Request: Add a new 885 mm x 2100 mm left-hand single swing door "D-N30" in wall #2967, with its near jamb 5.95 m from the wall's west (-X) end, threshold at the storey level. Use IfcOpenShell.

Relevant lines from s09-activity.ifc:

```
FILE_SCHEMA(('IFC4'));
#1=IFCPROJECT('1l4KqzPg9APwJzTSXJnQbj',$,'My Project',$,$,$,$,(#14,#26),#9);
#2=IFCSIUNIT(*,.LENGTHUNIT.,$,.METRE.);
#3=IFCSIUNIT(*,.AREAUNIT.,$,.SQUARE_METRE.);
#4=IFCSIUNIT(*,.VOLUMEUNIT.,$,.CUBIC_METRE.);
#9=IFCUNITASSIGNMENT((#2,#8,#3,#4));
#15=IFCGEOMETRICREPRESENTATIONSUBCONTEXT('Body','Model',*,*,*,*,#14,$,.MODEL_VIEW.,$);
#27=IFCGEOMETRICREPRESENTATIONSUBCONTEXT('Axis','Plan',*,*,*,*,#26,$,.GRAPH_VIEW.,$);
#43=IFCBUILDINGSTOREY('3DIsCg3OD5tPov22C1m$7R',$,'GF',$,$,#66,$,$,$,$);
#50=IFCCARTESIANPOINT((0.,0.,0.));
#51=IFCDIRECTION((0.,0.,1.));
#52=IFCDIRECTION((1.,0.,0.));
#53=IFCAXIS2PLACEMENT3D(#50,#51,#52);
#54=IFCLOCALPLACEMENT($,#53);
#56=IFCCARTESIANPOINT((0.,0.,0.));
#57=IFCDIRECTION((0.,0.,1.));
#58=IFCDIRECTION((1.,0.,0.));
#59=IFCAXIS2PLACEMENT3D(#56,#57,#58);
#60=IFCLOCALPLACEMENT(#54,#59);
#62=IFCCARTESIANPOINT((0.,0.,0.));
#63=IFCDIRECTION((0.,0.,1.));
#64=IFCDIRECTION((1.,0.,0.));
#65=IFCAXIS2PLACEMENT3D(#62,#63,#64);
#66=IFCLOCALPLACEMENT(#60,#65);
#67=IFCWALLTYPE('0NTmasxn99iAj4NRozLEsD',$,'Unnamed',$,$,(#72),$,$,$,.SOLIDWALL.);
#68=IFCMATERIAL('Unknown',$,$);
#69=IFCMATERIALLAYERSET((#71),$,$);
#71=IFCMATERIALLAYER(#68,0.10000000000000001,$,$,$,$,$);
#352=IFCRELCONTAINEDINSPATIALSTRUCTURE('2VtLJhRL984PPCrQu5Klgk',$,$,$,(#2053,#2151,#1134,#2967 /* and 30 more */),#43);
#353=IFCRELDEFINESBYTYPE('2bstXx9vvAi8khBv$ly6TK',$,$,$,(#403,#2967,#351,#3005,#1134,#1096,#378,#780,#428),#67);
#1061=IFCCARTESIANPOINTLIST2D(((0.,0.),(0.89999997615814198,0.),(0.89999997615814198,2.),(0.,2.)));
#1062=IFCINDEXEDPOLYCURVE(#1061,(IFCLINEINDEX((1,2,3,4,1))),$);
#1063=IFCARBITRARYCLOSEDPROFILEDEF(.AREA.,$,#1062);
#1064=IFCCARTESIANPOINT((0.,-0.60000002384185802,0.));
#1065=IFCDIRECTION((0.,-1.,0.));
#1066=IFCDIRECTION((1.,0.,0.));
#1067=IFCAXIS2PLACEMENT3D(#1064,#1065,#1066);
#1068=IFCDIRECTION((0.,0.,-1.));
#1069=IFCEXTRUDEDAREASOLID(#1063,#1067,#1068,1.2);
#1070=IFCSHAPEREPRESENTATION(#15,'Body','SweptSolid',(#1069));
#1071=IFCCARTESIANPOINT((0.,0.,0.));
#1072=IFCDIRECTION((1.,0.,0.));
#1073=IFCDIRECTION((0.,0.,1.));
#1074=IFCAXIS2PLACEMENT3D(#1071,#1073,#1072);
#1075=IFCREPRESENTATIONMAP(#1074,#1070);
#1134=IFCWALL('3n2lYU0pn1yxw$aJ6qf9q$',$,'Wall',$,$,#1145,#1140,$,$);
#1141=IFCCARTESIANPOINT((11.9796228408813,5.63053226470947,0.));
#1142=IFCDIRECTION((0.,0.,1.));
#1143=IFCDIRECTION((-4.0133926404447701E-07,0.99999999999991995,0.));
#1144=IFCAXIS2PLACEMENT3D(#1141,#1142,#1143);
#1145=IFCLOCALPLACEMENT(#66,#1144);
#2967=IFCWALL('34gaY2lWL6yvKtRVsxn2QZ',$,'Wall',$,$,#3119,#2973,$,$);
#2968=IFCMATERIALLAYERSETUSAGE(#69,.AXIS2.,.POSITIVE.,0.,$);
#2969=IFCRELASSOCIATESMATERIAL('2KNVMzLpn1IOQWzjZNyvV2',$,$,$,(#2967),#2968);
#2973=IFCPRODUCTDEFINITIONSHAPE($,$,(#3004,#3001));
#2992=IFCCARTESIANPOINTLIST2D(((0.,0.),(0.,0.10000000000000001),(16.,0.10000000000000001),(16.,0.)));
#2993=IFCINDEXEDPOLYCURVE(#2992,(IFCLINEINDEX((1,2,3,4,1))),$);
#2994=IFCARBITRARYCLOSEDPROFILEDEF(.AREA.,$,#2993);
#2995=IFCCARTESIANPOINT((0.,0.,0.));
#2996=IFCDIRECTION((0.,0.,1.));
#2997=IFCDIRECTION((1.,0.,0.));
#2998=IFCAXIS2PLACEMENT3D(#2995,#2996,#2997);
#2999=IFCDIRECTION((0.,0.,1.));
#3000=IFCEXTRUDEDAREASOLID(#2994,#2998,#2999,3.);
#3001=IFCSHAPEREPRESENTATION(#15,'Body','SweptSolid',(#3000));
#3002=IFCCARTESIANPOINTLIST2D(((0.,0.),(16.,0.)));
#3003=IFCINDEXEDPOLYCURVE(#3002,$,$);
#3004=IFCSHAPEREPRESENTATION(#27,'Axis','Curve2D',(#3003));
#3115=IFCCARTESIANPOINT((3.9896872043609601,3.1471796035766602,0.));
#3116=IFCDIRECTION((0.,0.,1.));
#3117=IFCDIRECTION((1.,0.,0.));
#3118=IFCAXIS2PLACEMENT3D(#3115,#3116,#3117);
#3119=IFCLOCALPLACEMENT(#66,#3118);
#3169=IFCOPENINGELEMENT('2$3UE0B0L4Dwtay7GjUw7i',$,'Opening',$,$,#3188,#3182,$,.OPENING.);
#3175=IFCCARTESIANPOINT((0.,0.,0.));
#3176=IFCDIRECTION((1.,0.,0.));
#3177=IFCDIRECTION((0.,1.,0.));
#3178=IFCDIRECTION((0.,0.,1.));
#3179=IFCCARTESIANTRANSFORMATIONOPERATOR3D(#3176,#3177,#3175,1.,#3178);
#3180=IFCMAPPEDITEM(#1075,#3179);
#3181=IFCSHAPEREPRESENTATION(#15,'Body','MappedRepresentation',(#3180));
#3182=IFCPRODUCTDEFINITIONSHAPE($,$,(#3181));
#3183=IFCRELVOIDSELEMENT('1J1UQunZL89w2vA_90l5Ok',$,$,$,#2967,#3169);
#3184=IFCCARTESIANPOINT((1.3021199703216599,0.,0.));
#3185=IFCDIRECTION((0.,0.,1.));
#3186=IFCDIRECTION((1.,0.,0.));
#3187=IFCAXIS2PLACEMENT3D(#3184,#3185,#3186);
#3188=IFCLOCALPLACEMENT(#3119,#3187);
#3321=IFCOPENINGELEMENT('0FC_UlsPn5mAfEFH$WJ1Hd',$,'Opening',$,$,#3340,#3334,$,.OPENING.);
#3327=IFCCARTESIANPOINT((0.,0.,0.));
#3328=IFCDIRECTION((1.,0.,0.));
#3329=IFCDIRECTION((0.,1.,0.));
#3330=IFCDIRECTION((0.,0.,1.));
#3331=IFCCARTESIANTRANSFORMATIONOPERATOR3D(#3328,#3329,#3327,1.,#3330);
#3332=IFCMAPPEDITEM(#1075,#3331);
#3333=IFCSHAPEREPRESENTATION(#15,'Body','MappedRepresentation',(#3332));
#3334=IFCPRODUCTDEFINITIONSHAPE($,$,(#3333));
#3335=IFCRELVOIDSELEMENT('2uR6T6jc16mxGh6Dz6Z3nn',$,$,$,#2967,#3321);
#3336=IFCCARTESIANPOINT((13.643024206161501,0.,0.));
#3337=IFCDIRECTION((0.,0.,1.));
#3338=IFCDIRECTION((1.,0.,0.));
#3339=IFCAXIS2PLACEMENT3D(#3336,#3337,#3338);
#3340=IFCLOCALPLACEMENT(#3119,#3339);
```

```python
import numpy as np
import ifcopenshell
import ifcopenshell.api.feature
import ifcopenshell.api.geometry
import ifcopenshell.api.root
import ifcopenshell.api.spatial
import ifcopenshell.geom
import ifcopenshell.util.element
import ifcopenshell.util.placement
import ifcopenshell.util.representation
import ifcopenshell.util.shape
import ifcopenshell.util.unit

model = ifcopenshell.open("s09-activity.ifc")
unit_scale = ifcopenshell.util.unit.calculate_unit_scale(model)
settings = ifcopenshell.geom.settings()


def volume(element):
    """Net volume in cubic metres, openings subtracted."""
    shape = ifcopenshell.geom.create_shape(settings, element)
    return ifcopenshell.util.shape.get_volume(shape.geometry)


wall = model.by_guid("34gaY2lWL6yvKtRVsxn2QZ")
storey = ifcopenshell.util.element.get_container(wall, ifc_class="IfcBuildingStorey")
context = ifcopenshell.util.representation.get_context(model, "Model", "Body", "MODEL_VIEW")
before = volume(wall)

width, height, from_end, sill = 0.885, 2.1, 5.95, 0.0  # metres

# The wall runs along its own X axis, and the end named is its -X end.
wall_shape = ifcopenshell.geom.create_shape(settings, wall)
x, y, z = ifcopenshell.util.shape.get_vertices(wall_shape.geometry).T
start = x.min() + from_end
face, thickness = float(y.min()), float(y.max() - y.min())
wall_matrix = ifcopenshell.util.placement.get_local_placement(wall.ObjectPlacement)
level = ifcopenshell.util.placement.get_local_placement(storey.ObjectPlacement)[2, 3]


def in_wall(x, y):
    """Placement at x, y metres in the wall's axes, at sill height."""
    matrix = wall_matrix.copy()
    matrix[:, 3] = wall_matrix @ np.array([x / unit_scale, y / unit_scale, 0.0, 1.0])
    matrix[2, 3] = level + sill / unit_scale
    return matrix


# Opening: a box that overshoots both wall faces by 50 mm.
opening = ifcopenshell.api.root.create_entity(model, ifc_class="IfcOpeningElement", predefined_type="OPENING")
box = ifcopenshell.api.geometry.add_wall_representation(
    model, context=context, length=width, height=height, thickness=thickness + 0.1
)
ifcopenshell.api.geometry.assign_representation(model, product=opening, representation=box)
ifcopenshell.api.geometry.edit_object_placement(model, product=opening, matrix=in_wall(start, face - 0.05), is_si=False)
ifcopenshell.api.feature.add_feature(model, feature=opening, element=wall)

door = ifcopenshell.api.root.create_entity(model, ifc_class="IfcDoor", name="D-N30", predefined_type="DOOR")
door.OverallWidth, door.OverallHeight = width / unit_scale, height / unit_scale
door.OperationType = "SINGLE_SWING_LEFT"
body = ifcopenshell.api.geometry.add_door_representation(
    model,
    context=context,
    overall_width=door.OverallWidth,
    overall_height=door.OverallHeight,
    operation_type="SINGLE_SWING_LEFT",
    lining_properties={"LiningDepth": thickness / unit_scale, "ThresholdDepth": thickness / unit_scale},
)
ifcopenshell.api.geometry.assign_representation(model, product=door, representation=body)
ifcopenshell.api.spatial.assign_container(model, products=[door], relating_structure=storey)
ifcopenshell.api.feature.add_filling(model, opening=opening, element=door)

# The lining spans the wall, so the door starts at the wall face.
ifcopenshell.api.geometry.edit_object_placement(model, product=door, matrix=in_wall(start, face), is_si=False)

after = volume(wall)

print(f"wall volume {before:.3f} -> {after:.3f} m3")

model.write("s09-activity-out.ifc")
```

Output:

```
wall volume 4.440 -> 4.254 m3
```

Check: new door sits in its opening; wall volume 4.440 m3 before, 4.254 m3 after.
